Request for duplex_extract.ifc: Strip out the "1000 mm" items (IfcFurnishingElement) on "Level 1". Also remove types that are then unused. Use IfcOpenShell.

First a look at what the model holds.

```python
import ifcopenshell
import ifcopenshell.util.element

model = ifcopenshell.open("duplex_extract.ifc")
print(model.schema)
storey = next(s for s in model.by_type("IfcBuildingStorey") if s.Name == "Level 1")
furniture = [e for e in ifcopenshell.util.element.get_decomposition(storey) if e.is_a("IfcFurnishingElement")]
seen = {}
for e in furniture:
    element_type = ifcopenshell.util.element.get_type(e)
    name = element_type.Name if element_type not in (None, e) else None
    seen[name] = seen.get(name, 0) + 1
for name, count in sorted(seen.items(), key=str):
    print(count, "x", name)
```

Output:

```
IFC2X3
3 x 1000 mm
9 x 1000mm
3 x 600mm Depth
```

```python
import ifcopenshell
import ifcopenshell.api.root
import ifcopenshell.util.element

model = ifcopenshell.open("duplex_extract.ifc")

storey = next(s for s in model.by_type("IfcBuildingStorey") if s.Name == "Level 1")
furniture = [e for e in ifcopenshell.util.element.get_decomposition(storey) if e.is_a("IfcFurnishingElement")]
targets = [e for e in furniture if (t := ifcopenshell.util.element.get_type(e)) not in (None, e) and t.Name == "1000 mm"]
types = {ifcopenshell.util.element.get_type(e) for e in targets} - {None, *targets}

for e in targets:
    ifcopenshell.api.root.remove_product(model, product=e)
print(len(targets), "removed")

unused = [t for t in types if not ifcopenshell.util.element.get_types(t)]
for t in unused:
    ifcopenshell.api.root.remove_product(model, product=t)
print(len(unused), "unused types removed")

model.write("duplex_extract_updated.ifc")
```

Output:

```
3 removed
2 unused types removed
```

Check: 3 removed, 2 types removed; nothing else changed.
